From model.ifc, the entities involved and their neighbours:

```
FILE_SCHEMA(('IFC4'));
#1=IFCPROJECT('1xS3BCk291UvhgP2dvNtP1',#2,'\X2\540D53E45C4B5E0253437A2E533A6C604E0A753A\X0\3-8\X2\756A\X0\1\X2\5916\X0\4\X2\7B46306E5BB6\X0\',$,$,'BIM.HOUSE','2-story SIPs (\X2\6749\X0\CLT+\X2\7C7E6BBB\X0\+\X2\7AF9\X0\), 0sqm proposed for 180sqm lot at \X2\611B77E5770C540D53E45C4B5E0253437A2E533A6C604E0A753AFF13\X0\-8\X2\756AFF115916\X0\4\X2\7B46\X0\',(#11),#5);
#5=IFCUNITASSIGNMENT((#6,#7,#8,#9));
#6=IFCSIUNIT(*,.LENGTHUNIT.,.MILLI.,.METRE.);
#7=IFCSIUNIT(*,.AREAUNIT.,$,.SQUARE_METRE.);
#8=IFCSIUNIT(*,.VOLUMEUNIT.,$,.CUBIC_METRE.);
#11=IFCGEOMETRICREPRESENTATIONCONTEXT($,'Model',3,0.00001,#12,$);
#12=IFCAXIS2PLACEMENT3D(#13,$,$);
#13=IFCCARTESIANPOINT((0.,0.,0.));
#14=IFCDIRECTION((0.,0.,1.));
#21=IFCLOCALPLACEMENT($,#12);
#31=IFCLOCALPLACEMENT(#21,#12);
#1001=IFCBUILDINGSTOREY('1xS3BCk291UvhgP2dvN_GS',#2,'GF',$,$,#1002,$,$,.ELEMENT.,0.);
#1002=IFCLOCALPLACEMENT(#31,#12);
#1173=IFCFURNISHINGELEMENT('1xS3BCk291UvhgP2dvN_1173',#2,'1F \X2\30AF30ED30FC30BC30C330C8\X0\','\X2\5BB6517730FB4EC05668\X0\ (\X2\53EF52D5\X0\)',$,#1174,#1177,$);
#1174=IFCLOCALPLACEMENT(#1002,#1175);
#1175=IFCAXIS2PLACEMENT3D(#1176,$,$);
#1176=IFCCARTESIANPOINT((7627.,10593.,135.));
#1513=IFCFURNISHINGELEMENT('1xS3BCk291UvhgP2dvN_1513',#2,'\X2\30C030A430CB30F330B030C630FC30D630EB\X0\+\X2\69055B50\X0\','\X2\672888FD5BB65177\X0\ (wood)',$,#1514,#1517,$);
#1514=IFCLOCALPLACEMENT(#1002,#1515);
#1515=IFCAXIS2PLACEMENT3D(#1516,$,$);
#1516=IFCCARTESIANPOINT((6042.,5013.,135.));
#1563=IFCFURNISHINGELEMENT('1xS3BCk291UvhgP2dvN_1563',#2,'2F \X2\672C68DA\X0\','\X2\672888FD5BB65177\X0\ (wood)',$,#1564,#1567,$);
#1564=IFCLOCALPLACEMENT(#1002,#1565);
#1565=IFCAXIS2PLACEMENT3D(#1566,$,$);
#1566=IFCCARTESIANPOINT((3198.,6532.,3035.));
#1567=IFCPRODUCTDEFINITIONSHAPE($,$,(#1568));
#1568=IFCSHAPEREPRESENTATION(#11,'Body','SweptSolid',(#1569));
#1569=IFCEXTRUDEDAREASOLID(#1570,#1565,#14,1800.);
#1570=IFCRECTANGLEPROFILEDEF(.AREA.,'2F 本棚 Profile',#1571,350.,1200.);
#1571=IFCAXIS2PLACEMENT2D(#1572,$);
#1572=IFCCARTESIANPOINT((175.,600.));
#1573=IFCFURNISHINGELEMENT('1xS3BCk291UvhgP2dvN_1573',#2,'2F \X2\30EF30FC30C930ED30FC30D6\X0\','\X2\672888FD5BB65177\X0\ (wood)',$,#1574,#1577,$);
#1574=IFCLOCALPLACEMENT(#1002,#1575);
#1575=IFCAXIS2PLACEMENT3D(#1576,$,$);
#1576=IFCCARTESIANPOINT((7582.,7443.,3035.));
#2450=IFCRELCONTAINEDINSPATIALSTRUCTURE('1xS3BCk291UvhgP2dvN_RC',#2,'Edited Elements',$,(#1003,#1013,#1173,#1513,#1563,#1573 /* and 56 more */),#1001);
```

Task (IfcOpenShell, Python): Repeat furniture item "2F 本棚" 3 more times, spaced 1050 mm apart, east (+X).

```python
import numpy as np
import ifcopenshell
import ifcopenshell.api.geometry
import ifcopenshell.api.root
import ifcopenshell.util.element
import ifcopenshell.util.placement

model = ifcopenshell.open("model.ifc")


def reuse_history(source, copy):
    """copy_class also copies each property set's owner history, people and application; keep the originals."""
    for rel in copy.IsDefinedBy:
        if rel.is_a("IfcRelDefinesByProperties") and (history := rel.RelatingPropertyDefinition.OwnerHistory):
            rel.RelatingPropertyDefinition.OwnerHistory = source.OwnerHistory
            ifcopenshell.util.element.remove_deep2(model, history)


source = model.by_id(1563)
base = ifcopenshell.util.placement.get_local_placement(source.ObjectPlacement)
step = np.array([1.0, 0.0, 0.0]) * 1050.0

for i in range(1, 4):
    copy = ifcopenshell.api.root.copy_class(model, product=source)
    copy.Representation = ifcopenshell.util.element.copy_deep(
        model, source.Representation, exclude=["IfcGeometricRepresentationContext", "IfcRepresentationMap"]
    )
    reuse_history(source, copy)
    matrix = base.copy()
    matrix[:3, 3] += i * step
    print("added at", matrix[:3, 3].round(3) + 0.0)
    ifcopenshell.api.geometry.edit_object_placement(model, product=copy, matrix=matrix, is_si=False)

model.write("model_updated.ifc")
```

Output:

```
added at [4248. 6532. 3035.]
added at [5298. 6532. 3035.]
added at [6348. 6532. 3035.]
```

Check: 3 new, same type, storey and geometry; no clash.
